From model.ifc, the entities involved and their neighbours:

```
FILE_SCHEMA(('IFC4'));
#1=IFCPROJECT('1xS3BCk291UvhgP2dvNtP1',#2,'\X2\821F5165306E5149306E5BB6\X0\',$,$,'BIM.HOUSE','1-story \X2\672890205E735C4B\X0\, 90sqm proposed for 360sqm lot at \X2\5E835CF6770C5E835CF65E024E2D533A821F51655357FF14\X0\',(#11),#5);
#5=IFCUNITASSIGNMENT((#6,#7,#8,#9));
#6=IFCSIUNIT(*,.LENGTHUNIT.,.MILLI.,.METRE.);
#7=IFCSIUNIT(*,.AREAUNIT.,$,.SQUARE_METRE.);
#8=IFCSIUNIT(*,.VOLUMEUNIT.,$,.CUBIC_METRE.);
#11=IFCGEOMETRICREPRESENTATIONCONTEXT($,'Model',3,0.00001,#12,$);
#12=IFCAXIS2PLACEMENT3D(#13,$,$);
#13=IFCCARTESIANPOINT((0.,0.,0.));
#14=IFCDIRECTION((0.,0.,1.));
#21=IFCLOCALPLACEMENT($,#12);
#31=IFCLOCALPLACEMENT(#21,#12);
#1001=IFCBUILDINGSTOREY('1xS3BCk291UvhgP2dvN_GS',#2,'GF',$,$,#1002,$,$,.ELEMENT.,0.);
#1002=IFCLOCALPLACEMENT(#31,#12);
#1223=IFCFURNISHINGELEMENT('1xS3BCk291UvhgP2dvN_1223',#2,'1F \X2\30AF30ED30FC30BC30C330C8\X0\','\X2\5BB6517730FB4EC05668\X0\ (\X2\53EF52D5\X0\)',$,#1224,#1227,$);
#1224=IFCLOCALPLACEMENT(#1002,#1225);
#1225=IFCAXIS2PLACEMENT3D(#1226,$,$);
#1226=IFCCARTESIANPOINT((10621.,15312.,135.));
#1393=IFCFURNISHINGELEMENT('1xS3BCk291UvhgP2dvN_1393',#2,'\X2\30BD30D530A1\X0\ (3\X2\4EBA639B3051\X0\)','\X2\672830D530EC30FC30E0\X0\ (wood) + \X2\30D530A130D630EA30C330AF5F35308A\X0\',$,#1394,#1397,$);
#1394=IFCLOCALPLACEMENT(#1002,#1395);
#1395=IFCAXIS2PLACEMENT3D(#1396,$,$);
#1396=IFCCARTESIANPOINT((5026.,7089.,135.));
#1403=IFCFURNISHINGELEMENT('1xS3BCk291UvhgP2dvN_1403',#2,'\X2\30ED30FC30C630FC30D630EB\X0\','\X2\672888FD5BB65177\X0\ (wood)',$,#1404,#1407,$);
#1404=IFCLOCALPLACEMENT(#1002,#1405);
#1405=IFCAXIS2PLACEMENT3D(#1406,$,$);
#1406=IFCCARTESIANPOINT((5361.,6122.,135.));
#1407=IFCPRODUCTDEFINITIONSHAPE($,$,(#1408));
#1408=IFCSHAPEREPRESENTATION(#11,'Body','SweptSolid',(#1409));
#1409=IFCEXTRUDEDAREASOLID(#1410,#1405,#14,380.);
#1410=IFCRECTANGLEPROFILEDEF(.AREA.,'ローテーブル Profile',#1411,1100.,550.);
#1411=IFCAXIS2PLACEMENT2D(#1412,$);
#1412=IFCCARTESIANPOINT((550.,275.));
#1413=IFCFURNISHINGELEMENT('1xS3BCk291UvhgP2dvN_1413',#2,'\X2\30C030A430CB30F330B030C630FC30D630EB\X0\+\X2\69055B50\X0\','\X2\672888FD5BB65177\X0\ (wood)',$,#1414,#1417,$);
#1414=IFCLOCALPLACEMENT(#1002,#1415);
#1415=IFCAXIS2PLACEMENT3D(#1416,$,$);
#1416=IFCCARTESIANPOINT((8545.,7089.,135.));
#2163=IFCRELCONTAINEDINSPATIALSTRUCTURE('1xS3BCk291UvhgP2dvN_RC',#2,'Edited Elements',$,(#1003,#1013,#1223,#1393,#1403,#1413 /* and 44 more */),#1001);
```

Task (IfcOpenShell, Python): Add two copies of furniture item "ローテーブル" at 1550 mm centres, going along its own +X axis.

```python
import ifcopenshell
import ifcopenshell.api.geometry
import ifcopenshell.api.root
import ifcopenshell.util.element
import ifcopenshell.util.placement
import ifcopenshell.util.unit

model = ifcopenshell.open("model.ifc")
unit_scale = ifcopenshell.util.unit.calculate_unit_scale(model)


def reuse_history(source, copy):
    """copy_class also copies each property set's owner history, people and application; keep the originals."""
    for rel in copy.IsDefinedBy:
        if rel.is_a("IfcRelDefinesByProperties") and (history := rel.RelatingPropertyDefinition.OwnerHistory):
            rel.RelatingPropertyDefinition.OwnerHistory = source.OwnerHistory
            ifcopenshell.util.element.remove_deep2(model, history)


source = model.by_guid("1xS3BCk291UvhgP2dvN_1403")
base = ifcopenshell.util.placement.get_local_placement(source.ObjectPlacement)
step = base[:3, 0] * 1.55 / unit_scale

for i in range(1, 3):
    copy = ifcopenshell.api.root.copy_class(model, product=source)
    copy.Representation = ifcopenshell.util.element.copy_deep(
        model, source.Representation, exclude=["IfcGeometricRepresentationContext", "IfcRepresentationMap"]
    )
    reuse_history(source, copy)
    matrix = base.copy()
    matrix[:3, 3] += i * step
    print("added at", matrix[:3, 3].round(3) + 0.0)
    ifcopenshell.api.geometry.edit_object_placement(model, product=copy, matrix=matrix, is_si=False)

model.write("model-out.ifc")
```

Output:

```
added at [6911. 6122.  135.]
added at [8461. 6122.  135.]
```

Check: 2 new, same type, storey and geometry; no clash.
